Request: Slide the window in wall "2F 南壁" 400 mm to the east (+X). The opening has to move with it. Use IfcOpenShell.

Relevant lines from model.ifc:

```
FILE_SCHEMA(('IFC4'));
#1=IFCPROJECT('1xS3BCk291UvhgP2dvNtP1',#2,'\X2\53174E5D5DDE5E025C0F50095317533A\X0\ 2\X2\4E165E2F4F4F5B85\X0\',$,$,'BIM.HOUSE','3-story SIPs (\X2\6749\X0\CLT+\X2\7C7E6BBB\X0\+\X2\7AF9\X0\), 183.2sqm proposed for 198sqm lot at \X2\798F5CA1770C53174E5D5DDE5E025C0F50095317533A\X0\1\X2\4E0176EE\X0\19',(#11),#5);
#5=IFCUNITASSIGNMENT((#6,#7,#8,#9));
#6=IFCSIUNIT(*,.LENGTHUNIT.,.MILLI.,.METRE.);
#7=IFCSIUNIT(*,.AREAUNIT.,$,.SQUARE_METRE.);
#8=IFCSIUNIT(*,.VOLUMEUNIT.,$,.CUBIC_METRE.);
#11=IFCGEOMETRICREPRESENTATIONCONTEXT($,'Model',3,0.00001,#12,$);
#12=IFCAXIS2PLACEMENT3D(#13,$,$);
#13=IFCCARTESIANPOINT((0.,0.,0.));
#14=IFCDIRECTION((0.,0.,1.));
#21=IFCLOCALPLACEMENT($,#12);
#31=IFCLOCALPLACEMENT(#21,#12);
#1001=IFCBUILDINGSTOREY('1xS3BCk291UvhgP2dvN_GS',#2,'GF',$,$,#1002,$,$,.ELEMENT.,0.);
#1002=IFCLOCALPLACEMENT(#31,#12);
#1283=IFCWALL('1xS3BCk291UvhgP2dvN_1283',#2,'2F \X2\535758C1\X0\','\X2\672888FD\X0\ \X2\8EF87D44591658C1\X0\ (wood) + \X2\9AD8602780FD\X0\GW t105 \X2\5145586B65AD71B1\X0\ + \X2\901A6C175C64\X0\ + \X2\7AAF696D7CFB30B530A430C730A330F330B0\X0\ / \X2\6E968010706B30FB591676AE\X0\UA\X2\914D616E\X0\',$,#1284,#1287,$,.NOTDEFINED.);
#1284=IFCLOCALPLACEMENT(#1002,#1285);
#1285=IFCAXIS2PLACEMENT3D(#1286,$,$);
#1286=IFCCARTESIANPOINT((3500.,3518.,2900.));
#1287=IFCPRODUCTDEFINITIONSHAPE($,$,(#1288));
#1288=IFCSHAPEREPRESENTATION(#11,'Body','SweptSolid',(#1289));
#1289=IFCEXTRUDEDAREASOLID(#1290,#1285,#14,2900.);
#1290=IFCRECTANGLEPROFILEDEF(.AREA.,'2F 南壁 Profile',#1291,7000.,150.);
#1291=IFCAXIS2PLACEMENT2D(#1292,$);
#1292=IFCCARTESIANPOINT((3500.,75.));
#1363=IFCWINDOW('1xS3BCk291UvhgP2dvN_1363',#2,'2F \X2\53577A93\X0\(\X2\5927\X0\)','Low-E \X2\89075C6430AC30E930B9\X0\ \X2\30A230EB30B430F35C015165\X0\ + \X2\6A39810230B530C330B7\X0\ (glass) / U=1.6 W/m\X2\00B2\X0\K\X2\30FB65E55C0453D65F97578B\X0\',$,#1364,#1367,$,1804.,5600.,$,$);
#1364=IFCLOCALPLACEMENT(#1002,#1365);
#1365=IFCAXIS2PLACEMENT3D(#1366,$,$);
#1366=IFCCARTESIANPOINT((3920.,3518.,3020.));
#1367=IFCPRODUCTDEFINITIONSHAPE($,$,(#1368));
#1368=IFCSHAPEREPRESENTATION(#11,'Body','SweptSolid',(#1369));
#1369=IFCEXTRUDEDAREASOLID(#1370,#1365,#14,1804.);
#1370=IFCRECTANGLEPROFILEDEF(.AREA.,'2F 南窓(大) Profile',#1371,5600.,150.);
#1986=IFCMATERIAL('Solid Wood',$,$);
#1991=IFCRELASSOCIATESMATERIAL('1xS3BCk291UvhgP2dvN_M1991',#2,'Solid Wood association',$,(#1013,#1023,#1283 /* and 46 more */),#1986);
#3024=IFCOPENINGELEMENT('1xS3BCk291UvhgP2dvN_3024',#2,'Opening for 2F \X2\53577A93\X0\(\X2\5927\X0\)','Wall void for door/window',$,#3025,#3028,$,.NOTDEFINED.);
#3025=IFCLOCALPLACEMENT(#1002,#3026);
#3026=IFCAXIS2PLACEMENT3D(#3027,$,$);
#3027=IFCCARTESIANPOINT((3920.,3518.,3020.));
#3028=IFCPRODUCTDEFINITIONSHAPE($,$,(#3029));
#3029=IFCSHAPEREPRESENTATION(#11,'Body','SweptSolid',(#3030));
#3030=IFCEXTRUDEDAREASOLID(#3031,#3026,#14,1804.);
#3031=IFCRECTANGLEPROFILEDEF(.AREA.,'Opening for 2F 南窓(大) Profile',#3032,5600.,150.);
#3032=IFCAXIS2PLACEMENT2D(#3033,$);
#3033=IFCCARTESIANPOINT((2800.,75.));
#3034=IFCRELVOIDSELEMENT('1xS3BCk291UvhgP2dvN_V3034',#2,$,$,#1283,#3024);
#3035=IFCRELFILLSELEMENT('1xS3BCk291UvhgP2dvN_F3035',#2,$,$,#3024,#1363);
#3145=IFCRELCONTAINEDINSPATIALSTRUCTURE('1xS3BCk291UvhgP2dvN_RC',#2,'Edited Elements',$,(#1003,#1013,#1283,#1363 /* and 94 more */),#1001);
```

```python
import ifcopenshell
import ifcopenshell.api.geometry
import ifcopenshell.util.placement
import ifcopenshell.util.unit

model = ifcopenshell.open("model.ifc")
unit_scale = ifcopenshell.util.unit.calculate_unit_scale(model)

window = model.by_id(1363)
opening = window.FillsVoids[0].RelatingOpeningElement
wall = opening.VoidsElements[0].RelatingBuildingElement

wall_matrix = ifcopenshell.util.placement.get_local_placement(wall.ObjectPlacement)
shift = wall_matrix[:3, 0] * 0.4 / unit_scale
before = ifcopenshell.util.placement.get_local_placement(window.ObjectPlacement)[:3, 3].copy()

# The window is not placed relative to its opening, so move both.
for product in (opening, window):
    matrix = ifcopenshell.util.placement.get_local_placement(product.ObjectPlacement)
    matrix[:3, 3] += shift
    ifcopenshell.api.geometry.edit_object_placement(model, product=product, matrix=matrix, is_si=False)

after = ifcopenshell.util.placement.get_local_placement(window.ObjectPlacement)[:3, 3]
print("window moved by", (after - before).round(3) + 0.0)

model.write("model_edited.ifc")
```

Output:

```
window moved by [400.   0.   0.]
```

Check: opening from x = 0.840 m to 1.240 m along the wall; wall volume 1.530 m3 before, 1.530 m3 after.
